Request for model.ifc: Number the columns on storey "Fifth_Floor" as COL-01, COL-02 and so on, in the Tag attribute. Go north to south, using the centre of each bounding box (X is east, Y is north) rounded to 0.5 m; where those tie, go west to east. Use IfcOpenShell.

First a look at what the model holds.

```python
import ifcopenshell
import ifcopenshell.util.element
import ifcopenshell.util.placement

model = ifcopenshell.open("model.ifc")
print(model.schema)
storey = next(s for s in model.by_type("IfcBuildingStorey") if s.Name == "Fifth_Floor")
columns = [e for e in ifcopenshell.util.element.get_decomposition(storey) if e.is_a("IfcColumn")]
for e in sorted(columns, key=lambda e: e.id()):
    origin = ifcopenshell.util.placement.get_local_placement(e.ObjectPlacement)[:3, 3]
    print(e.id(), e.Tag, e.Name, origin.round(2) + 0.0, sep=" | ")
```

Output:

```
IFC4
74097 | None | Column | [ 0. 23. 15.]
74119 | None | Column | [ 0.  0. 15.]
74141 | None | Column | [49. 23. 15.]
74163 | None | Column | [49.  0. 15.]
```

```python
import ifcopenshell
import ifcopenshell.geom
import ifcopenshell.util.element
import ifcopenshell.util.shape

model = ifcopenshell.open("model.ifc")
settings = ifcopenshell.geom.settings()
settings.set("use-world-coords", True)


def centre(element):
    shape = ifcopenshell.geom.create_shape(settings, element)
    return ifcopenshell.util.shape.get_bbox_centroid(shape.geometry)


storey = next(s for s in model.by_type("IfcBuildingStorey") if s.Name == "Fifth_Floor")
columns = [e for e in ifcopenshell.util.element.get_decomposition(storey) if e.is_a("IfcColumn")]

# Insertion points can sit at a corner or the storey origin, so sort by the geometry (in metres).
centres = {e: centre(e) for e in columns}
columns.sort(key=lambda e: (-round(centres[e][1] / 0.5), centres[e][0]))

for i, e in enumerate(columns, start=1):
    number = f"COL-{i:02d}"
    e.Tag = number
    print(e.id(), number)

model.write("model_updated.ifc")
```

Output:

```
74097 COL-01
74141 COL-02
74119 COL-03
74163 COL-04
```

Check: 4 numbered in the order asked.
